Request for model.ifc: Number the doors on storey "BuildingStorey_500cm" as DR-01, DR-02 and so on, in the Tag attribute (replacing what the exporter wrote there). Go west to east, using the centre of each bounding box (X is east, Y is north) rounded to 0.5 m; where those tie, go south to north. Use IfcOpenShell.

First a look at what the model holds.

```python
import ifcopenshell
import ifcopenshell.util.element
import ifcopenshell.util.placement

model = ifcopenshell.open("model.ifc")
print(model.schema)
storey = next(s for s in model.by_type("IfcBuildingStorey") if s.Name == "BuildingStorey_500cm")
doors = [e for e in ifcopenshell.util.element.get_decomposition(storey) if e.is_a("IfcDoor")]
for e in sorted(doors, key=lambda e: e.id()):
    origin = ifcopenshell.util.placement.get_local_placement(e.ObjectPlacement)[:3, 3]
    print(e.id(), e.Tag, e.Name, origin.round(2) + 0.0, sep=" | ")
```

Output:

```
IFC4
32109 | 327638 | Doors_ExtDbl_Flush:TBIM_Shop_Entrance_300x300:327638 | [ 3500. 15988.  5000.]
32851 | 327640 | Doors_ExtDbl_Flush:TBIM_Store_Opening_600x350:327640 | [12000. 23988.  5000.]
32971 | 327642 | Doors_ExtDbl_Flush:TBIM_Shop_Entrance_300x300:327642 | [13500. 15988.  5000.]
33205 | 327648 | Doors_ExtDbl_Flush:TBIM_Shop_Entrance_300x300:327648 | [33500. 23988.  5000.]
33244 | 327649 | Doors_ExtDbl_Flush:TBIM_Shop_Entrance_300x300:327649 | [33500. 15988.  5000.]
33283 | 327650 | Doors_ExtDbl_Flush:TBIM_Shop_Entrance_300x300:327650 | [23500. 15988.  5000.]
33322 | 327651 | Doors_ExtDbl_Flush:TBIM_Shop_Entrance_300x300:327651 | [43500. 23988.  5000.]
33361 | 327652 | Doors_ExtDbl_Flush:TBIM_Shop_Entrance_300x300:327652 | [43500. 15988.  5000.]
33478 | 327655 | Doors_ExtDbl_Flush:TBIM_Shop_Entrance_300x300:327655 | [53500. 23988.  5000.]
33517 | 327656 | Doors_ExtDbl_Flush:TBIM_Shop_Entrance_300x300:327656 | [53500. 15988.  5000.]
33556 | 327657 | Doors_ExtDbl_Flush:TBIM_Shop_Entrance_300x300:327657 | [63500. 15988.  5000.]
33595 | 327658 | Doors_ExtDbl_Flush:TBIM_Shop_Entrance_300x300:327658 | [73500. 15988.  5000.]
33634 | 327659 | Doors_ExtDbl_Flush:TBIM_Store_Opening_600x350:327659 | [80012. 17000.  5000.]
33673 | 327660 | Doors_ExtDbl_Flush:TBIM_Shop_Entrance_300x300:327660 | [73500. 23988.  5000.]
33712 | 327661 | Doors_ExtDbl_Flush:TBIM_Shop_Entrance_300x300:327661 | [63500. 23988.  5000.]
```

```python
import ifcopenshell
import ifcopenshell.geom
import ifcopenshell.util.element
import ifcopenshell.util.shape

model = ifcopenshell.open("model.ifc")
settings = ifcopenshell.geom.settings()
settings.set("use-world-coords", True)


def centre(element):
    shape = ifcopenshell.geom.create_shape(settings, element)
    return ifcopenshell.util.shape.get_bbox_centroid(shape.geometry)


storey = next(s for s in model.by_type("IfcBuildingStorey") if s.Name == "BuildingStorey_500cm")
doors = [e for e in ifcopenshell.util.element.get_decomposition(storey) if e.is_a("IfcDoor")]

# Insertion points can sit at a corner or the storey origin, so sort by the geometry (in metres).
centres = {e: centre(e) for e in doors}
doors.sort(key=lambda e: (round(centres[e][0] / 0.5), centres[e][1]))

for i, e in enumerate(doors, start=1):
    number = f"DR-{i:02d}"
    e.Tag = number
    print(e.id(), number)

model.write("model_edited.ifc")
```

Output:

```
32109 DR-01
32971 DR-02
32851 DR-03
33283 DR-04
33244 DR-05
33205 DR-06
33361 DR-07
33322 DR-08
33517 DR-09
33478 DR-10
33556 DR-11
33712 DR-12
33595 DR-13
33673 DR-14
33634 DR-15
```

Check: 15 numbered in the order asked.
